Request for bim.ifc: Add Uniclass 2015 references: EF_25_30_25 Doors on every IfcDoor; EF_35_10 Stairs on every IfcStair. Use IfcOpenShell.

First a look at what the model holds.

```python
import ifcopenshell

model = ifcopenshell.open("bim.ifc")
print(model.schema)
print("classifications:", [c.Name for c in model.by_type("IfcClassification")])
for ifc_class in ("IfcDoor", "IfcRoof", "IfcStair", "IfcWall", "IfcWindow"):
    print(ifc_class, len(model.by_type(ifc_class)))
```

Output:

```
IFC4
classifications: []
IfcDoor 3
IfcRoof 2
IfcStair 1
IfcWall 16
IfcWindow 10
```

```python
import ifcopenshell
import ifcopenshell.api.classification

model = ifcopenshell.open("bim.ifc")

system = ifcopenshell.api.classification.add_classification(model, classification="Uniclass 2015")

codes = {
    "IfcDoor": ("EF_25_30_25", "Doors"),
    "IfcStair": ("EF_35_10", "Stairs"),
}
for ifc_class, (code, name) in codes.items():
    products = model.by_type(ifc_class)
    ifcopenshell.api.classification.add_reference(
        model, products=products, classification=system, identification=code, name=name
    )
    print(code, len(products))

model.write("bim-out.ifc")
```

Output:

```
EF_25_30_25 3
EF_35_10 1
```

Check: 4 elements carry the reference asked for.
